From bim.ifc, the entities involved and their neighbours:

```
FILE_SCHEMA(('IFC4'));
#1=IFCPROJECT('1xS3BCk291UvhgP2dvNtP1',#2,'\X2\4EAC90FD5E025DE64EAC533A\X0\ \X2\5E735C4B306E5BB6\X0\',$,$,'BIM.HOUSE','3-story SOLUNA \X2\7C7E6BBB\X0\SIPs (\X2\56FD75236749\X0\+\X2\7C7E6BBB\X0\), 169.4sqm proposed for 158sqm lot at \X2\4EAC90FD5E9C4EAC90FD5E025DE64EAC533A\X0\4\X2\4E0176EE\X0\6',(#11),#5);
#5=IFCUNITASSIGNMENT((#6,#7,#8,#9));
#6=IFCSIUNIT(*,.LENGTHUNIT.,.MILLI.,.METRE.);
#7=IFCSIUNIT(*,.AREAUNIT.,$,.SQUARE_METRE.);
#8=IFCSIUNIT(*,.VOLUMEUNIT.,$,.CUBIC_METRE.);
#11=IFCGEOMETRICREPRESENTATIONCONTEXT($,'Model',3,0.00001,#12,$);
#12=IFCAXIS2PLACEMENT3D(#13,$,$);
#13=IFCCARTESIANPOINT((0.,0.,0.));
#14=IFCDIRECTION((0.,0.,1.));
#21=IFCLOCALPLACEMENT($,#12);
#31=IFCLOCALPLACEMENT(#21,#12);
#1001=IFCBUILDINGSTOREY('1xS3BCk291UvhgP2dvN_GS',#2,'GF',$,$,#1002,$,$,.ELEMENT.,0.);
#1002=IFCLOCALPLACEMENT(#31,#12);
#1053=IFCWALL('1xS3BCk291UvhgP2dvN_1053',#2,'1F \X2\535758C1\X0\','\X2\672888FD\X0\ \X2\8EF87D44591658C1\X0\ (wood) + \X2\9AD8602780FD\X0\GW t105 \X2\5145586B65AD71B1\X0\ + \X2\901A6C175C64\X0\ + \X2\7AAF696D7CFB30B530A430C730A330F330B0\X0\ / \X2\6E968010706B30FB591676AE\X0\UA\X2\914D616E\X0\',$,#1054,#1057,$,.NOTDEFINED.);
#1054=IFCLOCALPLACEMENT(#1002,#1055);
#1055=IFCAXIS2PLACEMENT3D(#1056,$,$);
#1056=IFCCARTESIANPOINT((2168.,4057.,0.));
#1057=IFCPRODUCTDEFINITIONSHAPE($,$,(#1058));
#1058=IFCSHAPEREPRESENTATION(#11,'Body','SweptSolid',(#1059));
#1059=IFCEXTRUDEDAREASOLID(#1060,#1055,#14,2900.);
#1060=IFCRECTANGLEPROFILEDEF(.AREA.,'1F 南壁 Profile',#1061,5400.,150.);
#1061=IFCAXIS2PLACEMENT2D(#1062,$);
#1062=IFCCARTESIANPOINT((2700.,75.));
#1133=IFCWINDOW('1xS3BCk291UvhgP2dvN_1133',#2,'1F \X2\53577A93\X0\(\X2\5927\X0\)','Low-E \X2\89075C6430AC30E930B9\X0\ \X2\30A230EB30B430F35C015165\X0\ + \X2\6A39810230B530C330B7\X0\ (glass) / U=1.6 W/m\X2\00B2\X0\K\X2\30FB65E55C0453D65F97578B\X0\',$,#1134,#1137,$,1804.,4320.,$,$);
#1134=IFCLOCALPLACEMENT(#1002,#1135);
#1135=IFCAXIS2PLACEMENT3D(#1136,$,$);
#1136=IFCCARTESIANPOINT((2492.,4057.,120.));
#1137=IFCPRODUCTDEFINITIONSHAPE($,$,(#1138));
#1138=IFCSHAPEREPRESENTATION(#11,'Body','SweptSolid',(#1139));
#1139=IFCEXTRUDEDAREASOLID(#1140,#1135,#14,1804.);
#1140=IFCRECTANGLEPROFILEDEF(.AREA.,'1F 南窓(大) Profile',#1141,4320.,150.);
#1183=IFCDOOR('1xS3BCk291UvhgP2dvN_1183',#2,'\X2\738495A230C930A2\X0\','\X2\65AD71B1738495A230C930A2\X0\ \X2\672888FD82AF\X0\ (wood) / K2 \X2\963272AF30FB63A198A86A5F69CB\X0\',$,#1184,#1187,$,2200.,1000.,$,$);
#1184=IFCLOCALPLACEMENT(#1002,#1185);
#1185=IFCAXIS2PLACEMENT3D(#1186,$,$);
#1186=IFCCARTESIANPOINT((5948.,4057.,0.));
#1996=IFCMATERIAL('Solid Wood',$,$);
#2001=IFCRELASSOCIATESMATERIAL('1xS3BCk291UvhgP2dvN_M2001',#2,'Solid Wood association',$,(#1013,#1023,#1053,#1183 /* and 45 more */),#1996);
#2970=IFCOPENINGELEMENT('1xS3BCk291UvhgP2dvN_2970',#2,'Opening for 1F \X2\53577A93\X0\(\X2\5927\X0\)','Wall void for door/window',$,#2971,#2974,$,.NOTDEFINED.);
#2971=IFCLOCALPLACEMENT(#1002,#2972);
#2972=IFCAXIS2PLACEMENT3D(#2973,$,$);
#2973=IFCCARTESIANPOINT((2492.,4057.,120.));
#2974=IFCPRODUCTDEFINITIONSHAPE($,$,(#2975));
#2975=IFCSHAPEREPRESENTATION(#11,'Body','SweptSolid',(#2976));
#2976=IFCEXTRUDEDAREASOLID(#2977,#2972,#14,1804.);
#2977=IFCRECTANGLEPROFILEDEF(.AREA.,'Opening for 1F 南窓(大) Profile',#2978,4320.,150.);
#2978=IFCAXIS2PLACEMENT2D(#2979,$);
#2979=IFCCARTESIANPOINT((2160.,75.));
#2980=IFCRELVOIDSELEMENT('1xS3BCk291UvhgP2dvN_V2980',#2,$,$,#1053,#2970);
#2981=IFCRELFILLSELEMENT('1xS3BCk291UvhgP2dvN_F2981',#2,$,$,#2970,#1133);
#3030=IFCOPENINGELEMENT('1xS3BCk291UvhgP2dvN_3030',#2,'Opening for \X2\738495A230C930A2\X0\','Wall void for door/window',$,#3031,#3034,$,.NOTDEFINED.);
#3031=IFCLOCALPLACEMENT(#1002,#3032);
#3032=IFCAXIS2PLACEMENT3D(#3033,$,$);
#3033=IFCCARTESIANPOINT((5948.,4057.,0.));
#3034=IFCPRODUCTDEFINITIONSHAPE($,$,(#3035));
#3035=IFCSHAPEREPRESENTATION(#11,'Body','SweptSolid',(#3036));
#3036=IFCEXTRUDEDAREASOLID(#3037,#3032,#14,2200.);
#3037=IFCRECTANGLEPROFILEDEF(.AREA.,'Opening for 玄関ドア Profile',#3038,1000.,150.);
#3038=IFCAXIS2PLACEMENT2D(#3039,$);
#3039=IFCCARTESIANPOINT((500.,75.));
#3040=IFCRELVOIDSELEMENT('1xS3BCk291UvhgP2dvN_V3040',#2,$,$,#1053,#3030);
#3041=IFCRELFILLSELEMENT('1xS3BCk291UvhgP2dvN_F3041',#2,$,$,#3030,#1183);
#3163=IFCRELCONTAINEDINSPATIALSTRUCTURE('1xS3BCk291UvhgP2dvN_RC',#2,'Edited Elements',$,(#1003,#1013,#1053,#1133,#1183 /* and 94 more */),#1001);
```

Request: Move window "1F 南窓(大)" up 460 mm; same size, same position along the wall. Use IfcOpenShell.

```python
import numpy as np
import ifcopenshell
import ifcopenshell.api.geometry
import ifcopenshell.util.placement
import ifcopenshell.util.unit

model = ifcopenshell.open("bim.ifc")
unit_scale = ifcopenshell.util.unit.calculate_unit_scale(model)

window = model.by_guid("1xS3BCk291UvhgP2dvN_1133")
opening = window.FillsVoids[0].RelatingOpeningElement
dz = 0.46 / unit_scale

shift = np.array([0.0, 0.0, dz])
# The window is not placed relative to its opening, so move both.
for product in (opening, window):
    matrix = ifcopenshell.util.placement.get_local_placement(product.ObjectPlacement)
    matrix[:3, 3] += shift
    ifcopenshell.api.geometry.edit_object_placement(model, product=product, matrix=matrix, is_si=False)

print(f"moved by {dz * unit_scale:+.3f} m")

model.write("bim_v2.ifc")
```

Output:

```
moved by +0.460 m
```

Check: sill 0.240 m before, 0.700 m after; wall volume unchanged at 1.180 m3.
